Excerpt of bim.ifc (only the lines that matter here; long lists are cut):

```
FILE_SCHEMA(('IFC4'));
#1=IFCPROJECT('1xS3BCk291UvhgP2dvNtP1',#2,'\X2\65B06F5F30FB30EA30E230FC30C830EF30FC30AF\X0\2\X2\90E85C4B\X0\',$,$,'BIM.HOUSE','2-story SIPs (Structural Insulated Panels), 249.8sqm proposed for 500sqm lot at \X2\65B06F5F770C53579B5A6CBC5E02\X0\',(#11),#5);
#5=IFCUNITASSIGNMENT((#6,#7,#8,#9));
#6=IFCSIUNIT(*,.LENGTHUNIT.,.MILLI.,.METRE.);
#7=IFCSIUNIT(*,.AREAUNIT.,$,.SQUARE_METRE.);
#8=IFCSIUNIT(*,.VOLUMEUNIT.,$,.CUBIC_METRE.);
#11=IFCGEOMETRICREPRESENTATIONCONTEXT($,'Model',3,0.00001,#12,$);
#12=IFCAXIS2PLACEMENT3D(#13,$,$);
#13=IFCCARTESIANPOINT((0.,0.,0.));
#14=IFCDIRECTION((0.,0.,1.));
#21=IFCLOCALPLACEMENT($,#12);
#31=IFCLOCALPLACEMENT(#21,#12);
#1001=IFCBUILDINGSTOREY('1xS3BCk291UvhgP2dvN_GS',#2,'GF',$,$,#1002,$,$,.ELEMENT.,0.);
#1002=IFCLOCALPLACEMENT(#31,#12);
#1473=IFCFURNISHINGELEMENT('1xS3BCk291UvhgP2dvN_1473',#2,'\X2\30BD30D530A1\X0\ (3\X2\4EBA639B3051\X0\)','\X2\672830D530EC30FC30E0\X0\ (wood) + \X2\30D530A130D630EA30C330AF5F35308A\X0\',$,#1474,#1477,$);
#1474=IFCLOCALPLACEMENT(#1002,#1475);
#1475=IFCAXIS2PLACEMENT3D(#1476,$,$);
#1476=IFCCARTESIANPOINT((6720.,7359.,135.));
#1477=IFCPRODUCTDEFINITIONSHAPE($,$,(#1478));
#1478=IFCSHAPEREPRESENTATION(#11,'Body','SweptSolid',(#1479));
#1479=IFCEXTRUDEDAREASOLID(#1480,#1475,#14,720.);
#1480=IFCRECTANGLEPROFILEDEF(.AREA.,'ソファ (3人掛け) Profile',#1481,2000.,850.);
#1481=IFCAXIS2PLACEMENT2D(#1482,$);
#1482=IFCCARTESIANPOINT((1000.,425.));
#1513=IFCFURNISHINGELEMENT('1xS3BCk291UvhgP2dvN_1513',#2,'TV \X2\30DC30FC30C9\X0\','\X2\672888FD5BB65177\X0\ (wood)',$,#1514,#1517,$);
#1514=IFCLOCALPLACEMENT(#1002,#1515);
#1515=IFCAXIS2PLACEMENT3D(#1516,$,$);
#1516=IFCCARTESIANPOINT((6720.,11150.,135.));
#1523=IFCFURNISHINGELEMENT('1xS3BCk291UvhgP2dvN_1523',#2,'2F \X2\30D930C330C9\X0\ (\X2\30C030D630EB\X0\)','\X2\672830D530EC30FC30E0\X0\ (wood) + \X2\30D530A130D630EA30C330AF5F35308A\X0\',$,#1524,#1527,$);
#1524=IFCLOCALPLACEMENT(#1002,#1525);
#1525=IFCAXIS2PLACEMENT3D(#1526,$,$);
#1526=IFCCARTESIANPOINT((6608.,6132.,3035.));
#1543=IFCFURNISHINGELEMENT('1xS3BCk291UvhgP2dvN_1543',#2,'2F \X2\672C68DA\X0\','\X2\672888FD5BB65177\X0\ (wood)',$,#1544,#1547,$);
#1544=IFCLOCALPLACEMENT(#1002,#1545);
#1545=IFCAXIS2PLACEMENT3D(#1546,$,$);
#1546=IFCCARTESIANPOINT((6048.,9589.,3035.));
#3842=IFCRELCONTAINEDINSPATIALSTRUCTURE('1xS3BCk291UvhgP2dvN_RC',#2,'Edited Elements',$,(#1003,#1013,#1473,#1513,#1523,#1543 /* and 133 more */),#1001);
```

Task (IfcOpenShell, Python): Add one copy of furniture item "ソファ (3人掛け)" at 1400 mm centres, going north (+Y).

```python
import numpy as np
import ifcopenshell
import ifcopenshell.api.geometry
import ifcopenshell.api.root
import ifcopenshell.util.element
import ifcopenshell.util.placement
import ifcopenshell.util.unit

model = ifcopenshell.open("bim.ifc")
unit_scale = ifcopenshell.util.unit.calculate_unit_scale(model)


def reuse_history(source, copy):
    """copy_class also copies each property set's owner history, people and application; keep the originals."""
    for rel in copy.IsDefinedBy:
        if rel.is_a("IfcRelDefinesByProperties") and (history := rel.RelatingPropertyDefinition.OwnerHistory):
            rel.RelatingPropertyDefinition.OwnerHistory = source.OwnerHistory
            ifcopenshell.util.element.remove_deep2(model, history)


source = model.by_guid("1xS3BCk291UvhgP2dvN_1473")
base = ifcopenshell.util.placement.get_local_placement(source.ObjectPlacement)
step = np.array([0.0, 1.0, 0.0]) * 1.4 / unit_scale

for i in range(1, 2):
    copy = ifcopenshell.api.root.copy_class(model, product=source)
    copy.Representation = ifcopenshell.util.element.copy_deep(
        model, source.Representation, exclude=["IfcGeometricRepresentationContext", "IfcRepresentationMap"]
    )
    reuse_history(source, copy)
    matrix = base.copy()
    matrix[:3, 3] += i * step
    print("added at", matrix[:3, 3].round(3) + 0.0)
    ifcopenshell.api.geometry.edit_object_placement(model, product=copy, matrix=matrix, is_si=False)

model.write("bim_rev.ifc")
```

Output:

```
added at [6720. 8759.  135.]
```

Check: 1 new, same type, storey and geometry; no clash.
